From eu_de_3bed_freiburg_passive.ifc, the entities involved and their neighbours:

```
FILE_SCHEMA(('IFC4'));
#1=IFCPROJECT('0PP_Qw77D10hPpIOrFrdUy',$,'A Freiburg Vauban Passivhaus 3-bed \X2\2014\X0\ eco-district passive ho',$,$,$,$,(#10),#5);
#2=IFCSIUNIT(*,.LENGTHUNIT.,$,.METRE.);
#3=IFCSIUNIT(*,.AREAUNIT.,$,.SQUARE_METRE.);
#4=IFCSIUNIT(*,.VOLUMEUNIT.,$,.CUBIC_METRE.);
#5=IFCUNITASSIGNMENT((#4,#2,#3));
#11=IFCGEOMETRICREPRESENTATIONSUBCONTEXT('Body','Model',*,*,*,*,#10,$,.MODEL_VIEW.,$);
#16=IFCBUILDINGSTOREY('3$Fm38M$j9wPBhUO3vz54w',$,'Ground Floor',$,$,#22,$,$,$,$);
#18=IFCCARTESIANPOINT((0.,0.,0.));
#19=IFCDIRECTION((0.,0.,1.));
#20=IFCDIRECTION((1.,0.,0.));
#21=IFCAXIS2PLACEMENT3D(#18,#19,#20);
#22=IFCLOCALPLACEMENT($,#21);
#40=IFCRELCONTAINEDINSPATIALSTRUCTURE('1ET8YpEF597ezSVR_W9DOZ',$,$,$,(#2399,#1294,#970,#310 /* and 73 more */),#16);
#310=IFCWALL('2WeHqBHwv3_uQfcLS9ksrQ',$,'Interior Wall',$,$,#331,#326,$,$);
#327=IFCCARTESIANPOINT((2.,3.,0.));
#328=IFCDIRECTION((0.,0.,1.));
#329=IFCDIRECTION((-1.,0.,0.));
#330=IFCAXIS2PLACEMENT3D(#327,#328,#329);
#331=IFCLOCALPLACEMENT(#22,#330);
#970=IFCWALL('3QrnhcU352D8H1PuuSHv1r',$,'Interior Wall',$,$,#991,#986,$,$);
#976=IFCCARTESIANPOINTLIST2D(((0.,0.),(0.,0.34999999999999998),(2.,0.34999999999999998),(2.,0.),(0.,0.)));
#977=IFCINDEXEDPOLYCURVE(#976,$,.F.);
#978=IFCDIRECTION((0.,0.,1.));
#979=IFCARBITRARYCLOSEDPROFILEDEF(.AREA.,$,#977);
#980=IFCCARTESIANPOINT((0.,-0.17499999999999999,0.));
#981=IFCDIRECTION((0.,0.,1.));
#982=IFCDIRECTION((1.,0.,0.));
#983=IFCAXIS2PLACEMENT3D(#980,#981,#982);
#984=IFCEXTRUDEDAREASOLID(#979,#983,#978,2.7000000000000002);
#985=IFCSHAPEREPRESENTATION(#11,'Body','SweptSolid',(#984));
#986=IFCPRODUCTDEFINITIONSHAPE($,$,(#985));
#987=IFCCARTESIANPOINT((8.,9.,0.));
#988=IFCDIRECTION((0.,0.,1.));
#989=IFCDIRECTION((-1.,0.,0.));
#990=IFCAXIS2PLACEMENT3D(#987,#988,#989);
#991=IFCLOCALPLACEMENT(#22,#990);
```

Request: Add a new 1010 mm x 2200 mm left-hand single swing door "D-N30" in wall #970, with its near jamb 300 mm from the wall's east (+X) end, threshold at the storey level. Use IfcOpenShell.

```python
import numpy as np
import ifcopenshell
import ifcopenshell.api.feature
import ifcopenshell.api.geometry
import ifcopenshell.api.root
import ifcopenshell.api.spatial
import ifcopenshell.geom
import ifcopenshell.util.element
import ifcopenshell.util.placement
import ifcopenshell.util.representation
import ifcopenshell.util.shape
import ifcopenshell.util.unit

model = ifcopenshell.open("eu_de_3bed_freiburg_passive.ifc")
unit_scale = ifcopenshell.util.unit.calculate_unit_scale(model)
settings = ifcopenshell.geom.settings()


def volume(element):
    """Net volume in cubic metres, openings subtracted."""
    shape = ifcopenshell.geom.create_shape(settings, element)
    return ifcopenshell.util.shape.get_volume(shape.geometry)


wall = model.by_guid("3QrnhcU352D8H1PuuSHv1r")
storey = ifcopenshell.util.element.get_container(wall, ifc_class="IfcBuildingStorey")
context = ifcopenshell.util.representation.get_context(model, "Model", "Body", "MODEL_VIEW")
before = volume(wall)

width, height, from_end, sill = 1.01, 2.2, 0.3, 0.0  # metres

# The wall runs along its own X axis, and the end named is its -X end.
wall_shape = ifcopenshell.geom.create_shape(settings, wall)
x, y, z = ifcopenshell.util.shape.get_vertices(wall_shape.geometry).T
start = x.min() + from_end
face, thickness = float(y.min()), float(y.max() - y.min())
wall_matrix = ifcopenshell.util.placement.get_local_placement(wall.ObjectPlacement)
level = ifcopenshell.util.placement.get_local_placement(storey.ObjectPlacement)[2, 3]


def in_wall(x, y):
    """Placement at x, y metres in the wall's axes, at sill height."""
    matrix = wall_matrix.copy()
    matrix[:, 3] = wall_matrix @ np.array([x / unit_scale, y / unit_scale, 0.0, 1.0])
    matrix[2, 3] = level + sill / unit_scale
    return matrix


# Opening: a box that overshoots both wall faces by 50 mm.
opening = ifcopenshell.api.root.create_entity(model, ifc_class="IfcOpeningElement", predefined_type="OPENING")
box = ifcopenshell.api.geometry.add_wall_representation(
    model, context=context, length=width, height=height, thickness=thickness + 0.1
)
ifcopenshell.api.geometry.assign_representation(model, product=opening, representation=box)
ifcopenshell.api.geometry.edit_object_placement(model, product=opening, matrix=in_wall(start, face - 0.05), is_si=False)
ifcopenshell.api.feature.add_feature(model, feature=opening, element=wall)

door = ifcopenshell.api.root.create_entity(model, ifc_class="IfcDoor", name="D-N30", predefined_type="DOOR")
door.OverallWidth, door.OverallHeight = width / unit_scale, height / unit_scale
door.OperationType = "SINGLE_SWING_LEFT"
body = ifcopenshell.api.geometry.add_door_representation(
    model,
    context=context,
    overall_width=door.OverallWidth,
    overall_height=door.OverallHeight,
    operation_type="SINGLE_SWING_LEFT",
    lining_properties={"LiningDepth": thickness / unit_scale, "ThresholdDepth": thickness / unit_scale},
)
ifcopenshell.api.geometry.assign_representation(model, product=door, representation=body)
ifcopenshell.api.spatial.assign_container(model, products=[door], relating_structure=storey)
ifcopenshell.api.feature.add_filling(model, opening=opening, element=door)

# The lining spans the wall, so the door starts at the wall face.
ifcopenshell.api.geometry.edit_object_placement(model, product=door, matrix=in_wall(start, face), is_si=False)

after = volume(wall)

print(f"wall volume {before:.3f} -> {after:.3f} m3")

model.write("eu_de_3bed_freiburg_passive-out.ifc")
```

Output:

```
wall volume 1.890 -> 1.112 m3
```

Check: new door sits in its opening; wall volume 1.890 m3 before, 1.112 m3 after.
